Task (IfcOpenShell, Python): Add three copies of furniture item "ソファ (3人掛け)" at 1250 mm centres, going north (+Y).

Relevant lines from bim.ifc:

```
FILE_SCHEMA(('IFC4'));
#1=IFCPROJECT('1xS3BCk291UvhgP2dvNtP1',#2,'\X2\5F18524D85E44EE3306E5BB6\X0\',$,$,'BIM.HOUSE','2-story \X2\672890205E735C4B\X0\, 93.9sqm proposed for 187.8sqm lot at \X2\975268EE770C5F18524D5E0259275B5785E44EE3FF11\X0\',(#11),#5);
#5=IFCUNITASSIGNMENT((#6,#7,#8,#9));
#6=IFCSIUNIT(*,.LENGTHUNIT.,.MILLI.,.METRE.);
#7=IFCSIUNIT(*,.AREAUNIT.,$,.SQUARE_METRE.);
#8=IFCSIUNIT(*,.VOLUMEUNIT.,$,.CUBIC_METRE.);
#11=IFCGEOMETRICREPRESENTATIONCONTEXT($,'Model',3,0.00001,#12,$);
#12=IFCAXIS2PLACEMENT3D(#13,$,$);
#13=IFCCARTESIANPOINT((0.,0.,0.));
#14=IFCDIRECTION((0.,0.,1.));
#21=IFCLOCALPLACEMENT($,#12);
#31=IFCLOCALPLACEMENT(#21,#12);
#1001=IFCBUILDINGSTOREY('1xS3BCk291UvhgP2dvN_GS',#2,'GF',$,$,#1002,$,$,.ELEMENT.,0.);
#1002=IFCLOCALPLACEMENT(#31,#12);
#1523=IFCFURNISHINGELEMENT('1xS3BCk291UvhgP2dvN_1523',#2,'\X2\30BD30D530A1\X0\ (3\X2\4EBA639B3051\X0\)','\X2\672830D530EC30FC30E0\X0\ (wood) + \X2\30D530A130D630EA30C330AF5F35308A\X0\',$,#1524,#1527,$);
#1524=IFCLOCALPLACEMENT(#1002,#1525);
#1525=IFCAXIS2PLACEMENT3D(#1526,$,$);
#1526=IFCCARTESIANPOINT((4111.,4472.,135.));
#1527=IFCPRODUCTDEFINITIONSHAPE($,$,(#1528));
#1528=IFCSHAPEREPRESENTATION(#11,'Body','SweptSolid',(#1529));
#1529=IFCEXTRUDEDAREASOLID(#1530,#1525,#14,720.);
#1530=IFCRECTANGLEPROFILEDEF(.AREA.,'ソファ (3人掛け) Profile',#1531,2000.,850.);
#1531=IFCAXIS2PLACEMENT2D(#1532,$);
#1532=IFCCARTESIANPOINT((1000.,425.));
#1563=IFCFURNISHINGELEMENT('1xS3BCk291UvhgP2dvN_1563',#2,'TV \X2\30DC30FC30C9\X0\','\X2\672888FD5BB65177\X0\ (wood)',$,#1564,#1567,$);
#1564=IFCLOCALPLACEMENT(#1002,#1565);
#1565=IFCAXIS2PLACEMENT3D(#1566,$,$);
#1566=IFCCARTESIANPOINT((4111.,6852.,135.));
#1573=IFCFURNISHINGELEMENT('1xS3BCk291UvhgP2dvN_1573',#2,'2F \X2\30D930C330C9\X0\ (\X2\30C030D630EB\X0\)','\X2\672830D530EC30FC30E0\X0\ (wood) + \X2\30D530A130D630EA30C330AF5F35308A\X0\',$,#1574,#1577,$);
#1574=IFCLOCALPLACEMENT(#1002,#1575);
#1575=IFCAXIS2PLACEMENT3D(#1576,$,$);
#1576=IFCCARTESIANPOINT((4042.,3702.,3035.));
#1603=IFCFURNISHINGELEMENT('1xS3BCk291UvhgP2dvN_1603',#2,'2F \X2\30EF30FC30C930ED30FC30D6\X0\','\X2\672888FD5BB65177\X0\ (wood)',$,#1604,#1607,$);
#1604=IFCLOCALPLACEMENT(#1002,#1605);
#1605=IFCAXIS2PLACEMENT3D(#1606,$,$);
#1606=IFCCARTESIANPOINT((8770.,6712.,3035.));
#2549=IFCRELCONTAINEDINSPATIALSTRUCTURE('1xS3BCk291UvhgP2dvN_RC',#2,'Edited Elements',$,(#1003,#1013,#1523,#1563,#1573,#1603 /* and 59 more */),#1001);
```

```python
import numpy as np
import ifcopenshell
import ifcopenshell.api.geometry
import ifcopenshell.api.root
import ifcopenshell.util.element
import ifcopenshell.util.placement

model = ifcopenshell.open("bim.ifc")


def reuse_history(source, copy):
    """copy_class also copies each property set's owner history, people and application; keep the originals."""
    for rel in copy.IsDefinedBy:
        if rel.is_a("IfcRelDefinesByProperties") and (history := rel.RelatingPropertyDefinition.OwnerHistory):
            rel.RelatingPropertyDefinition.OwnerHistory = source.OwnerHistory
            ifcopenshell.util.element.remove_deep2(model, history)


source = model.by_guid("1xS3BCk291UvhgP2dvN_1523")
base = ifcopenshell.util.placement.get_local_placement(source.ObjectPlacement)
step = np.array([0.0, 1.0, 0.0]) * 1250.0

for i in range(1, 4):
    copy = ifcopenshell.api.root.copy_class(model, product=source)
    copy.Representation = ifcopenshell.util.element.copy_deep(
        model, source.Representation, exclude=["IfcGeometricRepresentationContext", "IfcRepresentationMap"]
    )
    reuse_history(source, copy)
    matrix = base.copy()
    matrix[:3, 3] += i * step
    print("added at", matrix[:3, 3].round(3) + 0.0)
    ifcopenshell.api.geometry.edit_object_placement(model, product=copy, matrix=matrix, is_si=False)

model.write("bim_edited.ifc")
```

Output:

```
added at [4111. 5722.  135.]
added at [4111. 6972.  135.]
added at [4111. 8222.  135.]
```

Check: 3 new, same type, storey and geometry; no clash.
